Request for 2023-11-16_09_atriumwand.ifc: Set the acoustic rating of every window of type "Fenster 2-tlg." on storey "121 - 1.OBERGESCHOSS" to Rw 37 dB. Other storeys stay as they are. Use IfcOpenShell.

First a look at what the model holds.

```python
import ifcopenshell
import ifcopenshell.util.element

model = ifcopenshell.open("2023-11-16_09_atriumwand.ifc")
print(model.schema)
storey = next(s for s in model.by_type("IfcBuildingStorey") if s.Name == "121 - 1.OBERGESCHOSS")
windows = [e for e in ifcopenshell.util.element.get_decomposition(storey) if e.is_a("IfcWindow")]
seen = {}
for e in windows:
    element_type = ifcopenshell.util.element.get_type(e)
    key = (element_type.Name if element_type != e and element_type else None, ifcopenshell.util.element.get_pset(e, "Pset_WindowCommon", "AcousticRating"))
    seen[key] = seen.get(key, 0) + 1
for (name, value), count in sorted(seen.items(), key=str):
    print(count, "x", name, "|", value)
```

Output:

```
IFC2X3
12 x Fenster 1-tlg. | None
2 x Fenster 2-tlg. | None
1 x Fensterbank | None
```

```python
import ifcopenshell
import ifcopenshell.api.pset
import ifcopenshell.util.element

model = ifcopenshell.open("2023-11-16_09_atriumwand.ifc")

storey = next(s for s in model.by_type("IfcBuildingStorey") if s.Name == "121 - 1.OBERGESCHOSS")
windows = [e for e in ifcopenshell.util.element.get_decomposition(storey) if e.is_a("IfcWindow")]

count = 0
for e in windows:
    element_type = ifcopenshell.util.element.get_type(e)
    if element_type in (None, e) or element_type.Name != "Fenster 2-tlg.":
        continue
    # add_pset returns the element's existing set when there is one.
    pset = ifcopenshell.api.pset.add_pset(model, product=e, name="Pset_WindowCommon")
    ifcopenshell.api.pset.edit_pset(model, pset=pset, properties={"AcousticRating": "Rw 37 dB"})
    count += 1

print(count, "windows updated")

model.write("2023-11-16_09_atriumwand_edited.ifc")
```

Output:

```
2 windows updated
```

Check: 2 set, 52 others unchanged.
